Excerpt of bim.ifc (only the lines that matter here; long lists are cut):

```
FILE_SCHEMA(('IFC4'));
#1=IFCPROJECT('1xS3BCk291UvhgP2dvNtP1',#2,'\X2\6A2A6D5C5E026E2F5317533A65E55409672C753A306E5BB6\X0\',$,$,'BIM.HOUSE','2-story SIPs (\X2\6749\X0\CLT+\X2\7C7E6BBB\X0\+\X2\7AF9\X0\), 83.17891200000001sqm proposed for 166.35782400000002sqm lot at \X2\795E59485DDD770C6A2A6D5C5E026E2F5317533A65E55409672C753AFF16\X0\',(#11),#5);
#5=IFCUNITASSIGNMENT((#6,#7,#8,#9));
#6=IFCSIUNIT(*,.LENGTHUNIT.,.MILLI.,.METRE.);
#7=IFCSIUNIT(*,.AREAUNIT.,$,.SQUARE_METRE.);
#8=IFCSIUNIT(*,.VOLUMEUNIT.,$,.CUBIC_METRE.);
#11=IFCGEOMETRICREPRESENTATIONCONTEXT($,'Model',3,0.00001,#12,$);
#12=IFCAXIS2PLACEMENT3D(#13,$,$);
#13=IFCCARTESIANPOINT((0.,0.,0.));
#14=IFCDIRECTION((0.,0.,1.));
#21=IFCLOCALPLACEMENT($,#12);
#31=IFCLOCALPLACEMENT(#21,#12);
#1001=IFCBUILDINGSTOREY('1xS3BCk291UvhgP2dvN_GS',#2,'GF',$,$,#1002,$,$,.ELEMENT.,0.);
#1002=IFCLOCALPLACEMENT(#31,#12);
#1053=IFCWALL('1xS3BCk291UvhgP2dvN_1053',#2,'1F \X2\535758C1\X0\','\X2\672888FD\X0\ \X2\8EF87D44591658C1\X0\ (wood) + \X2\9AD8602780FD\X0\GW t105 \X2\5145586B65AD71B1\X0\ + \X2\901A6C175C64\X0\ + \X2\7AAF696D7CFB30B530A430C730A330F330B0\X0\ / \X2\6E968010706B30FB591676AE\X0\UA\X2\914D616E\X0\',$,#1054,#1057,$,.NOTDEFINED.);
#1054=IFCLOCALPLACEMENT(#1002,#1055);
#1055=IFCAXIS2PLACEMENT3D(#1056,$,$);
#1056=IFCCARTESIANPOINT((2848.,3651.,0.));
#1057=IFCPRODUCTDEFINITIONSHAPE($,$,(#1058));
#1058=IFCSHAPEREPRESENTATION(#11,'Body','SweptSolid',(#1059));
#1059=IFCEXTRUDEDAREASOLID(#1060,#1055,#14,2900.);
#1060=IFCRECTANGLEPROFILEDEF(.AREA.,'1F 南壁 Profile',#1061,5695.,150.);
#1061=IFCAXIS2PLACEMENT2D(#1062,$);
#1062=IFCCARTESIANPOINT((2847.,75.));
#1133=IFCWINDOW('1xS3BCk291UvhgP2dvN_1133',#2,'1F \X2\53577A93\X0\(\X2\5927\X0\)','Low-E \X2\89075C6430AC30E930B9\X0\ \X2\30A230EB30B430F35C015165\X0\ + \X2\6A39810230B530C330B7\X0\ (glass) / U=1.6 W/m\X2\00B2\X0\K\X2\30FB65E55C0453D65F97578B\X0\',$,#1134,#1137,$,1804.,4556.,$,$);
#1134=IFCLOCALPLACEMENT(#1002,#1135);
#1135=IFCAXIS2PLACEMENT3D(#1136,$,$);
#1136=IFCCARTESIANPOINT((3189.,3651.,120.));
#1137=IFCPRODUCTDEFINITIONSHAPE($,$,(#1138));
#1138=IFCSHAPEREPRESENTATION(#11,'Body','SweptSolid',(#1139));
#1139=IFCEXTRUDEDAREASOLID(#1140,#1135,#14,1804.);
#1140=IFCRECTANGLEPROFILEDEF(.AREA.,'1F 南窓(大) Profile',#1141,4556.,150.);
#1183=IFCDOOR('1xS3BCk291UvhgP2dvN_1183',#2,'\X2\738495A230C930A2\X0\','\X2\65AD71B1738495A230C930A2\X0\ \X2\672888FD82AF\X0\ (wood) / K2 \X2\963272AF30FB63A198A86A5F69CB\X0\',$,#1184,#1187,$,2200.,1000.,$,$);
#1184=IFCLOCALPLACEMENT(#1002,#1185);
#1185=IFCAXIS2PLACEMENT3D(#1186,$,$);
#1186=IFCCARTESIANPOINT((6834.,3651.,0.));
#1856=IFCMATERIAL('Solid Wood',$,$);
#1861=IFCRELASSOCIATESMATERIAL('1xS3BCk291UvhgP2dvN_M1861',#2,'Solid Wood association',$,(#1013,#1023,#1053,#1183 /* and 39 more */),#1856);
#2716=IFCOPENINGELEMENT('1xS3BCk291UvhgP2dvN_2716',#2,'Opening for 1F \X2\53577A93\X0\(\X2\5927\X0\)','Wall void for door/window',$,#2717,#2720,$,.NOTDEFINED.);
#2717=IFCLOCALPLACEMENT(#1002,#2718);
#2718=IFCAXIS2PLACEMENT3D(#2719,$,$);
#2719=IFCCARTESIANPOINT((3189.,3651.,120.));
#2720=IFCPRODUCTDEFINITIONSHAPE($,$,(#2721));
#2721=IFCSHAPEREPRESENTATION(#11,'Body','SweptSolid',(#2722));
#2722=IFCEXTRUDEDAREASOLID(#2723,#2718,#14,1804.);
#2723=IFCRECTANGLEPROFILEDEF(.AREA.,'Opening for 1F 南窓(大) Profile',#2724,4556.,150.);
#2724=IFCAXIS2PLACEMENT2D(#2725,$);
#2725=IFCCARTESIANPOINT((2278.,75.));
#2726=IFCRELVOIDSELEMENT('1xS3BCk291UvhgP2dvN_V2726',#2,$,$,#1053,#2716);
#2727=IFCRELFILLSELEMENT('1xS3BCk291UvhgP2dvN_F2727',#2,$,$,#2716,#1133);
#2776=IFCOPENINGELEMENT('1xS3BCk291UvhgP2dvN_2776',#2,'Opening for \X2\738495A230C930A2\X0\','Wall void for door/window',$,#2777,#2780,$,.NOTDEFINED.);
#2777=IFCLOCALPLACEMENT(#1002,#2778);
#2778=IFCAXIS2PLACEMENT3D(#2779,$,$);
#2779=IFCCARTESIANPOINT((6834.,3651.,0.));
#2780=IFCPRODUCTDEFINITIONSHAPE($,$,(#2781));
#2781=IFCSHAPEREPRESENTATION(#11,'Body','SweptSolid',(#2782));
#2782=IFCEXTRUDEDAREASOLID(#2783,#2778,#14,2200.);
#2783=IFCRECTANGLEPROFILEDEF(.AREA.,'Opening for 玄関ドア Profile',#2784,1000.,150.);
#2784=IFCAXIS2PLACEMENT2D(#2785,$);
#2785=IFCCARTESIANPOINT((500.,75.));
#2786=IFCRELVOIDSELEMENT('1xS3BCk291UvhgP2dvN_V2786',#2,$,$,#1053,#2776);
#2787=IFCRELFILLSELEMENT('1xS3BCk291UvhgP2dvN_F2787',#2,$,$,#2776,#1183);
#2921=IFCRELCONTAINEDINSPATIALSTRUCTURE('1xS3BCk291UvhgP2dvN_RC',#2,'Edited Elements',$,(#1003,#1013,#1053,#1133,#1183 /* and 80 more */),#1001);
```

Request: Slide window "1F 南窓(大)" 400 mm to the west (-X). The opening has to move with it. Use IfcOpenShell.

```python
import ifcopenshell
import ifcopenshell.api.geometry
import ifcopenshell.util.placement

model = ifcopenshell.open("bim.ifc")

window = model.by_id(1133)
opening = window.FillsVoids[0].RelatingOpeningElement
wall = opening.VoidsElements[0].RelatingBuildingElement

wall_matrix = ifcopenshell.util.placement.get_local_placement(wall.ObjectPlacement)
shift = wall_matrix[:3, 0] * -400.0
before = ifcopenshell.util.placement.get_local_placement(window.ObjectPlacement)[:3, 3].copy()

# The window is not placed relative to its opening, so move both.
for product in (opening, window):
    matrix = ifcopenshell.util.placement.get_local_placement(product.ObjectPlacement)
    matrix[:3, 3] += shift
    ifcopenshell.api.geometry.edit_object_placement(model, product=product, matrix=matrix, is_si=False)

after = ifcopenshell.util.placement.get_local_placement(window.ObjectPlacement)[:3, 3]
print("window moved by", (after - before).round(3) + 0.0)

model.write("bim_rev.ifc")
```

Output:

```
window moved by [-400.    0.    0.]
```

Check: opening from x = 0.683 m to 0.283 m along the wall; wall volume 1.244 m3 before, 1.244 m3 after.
